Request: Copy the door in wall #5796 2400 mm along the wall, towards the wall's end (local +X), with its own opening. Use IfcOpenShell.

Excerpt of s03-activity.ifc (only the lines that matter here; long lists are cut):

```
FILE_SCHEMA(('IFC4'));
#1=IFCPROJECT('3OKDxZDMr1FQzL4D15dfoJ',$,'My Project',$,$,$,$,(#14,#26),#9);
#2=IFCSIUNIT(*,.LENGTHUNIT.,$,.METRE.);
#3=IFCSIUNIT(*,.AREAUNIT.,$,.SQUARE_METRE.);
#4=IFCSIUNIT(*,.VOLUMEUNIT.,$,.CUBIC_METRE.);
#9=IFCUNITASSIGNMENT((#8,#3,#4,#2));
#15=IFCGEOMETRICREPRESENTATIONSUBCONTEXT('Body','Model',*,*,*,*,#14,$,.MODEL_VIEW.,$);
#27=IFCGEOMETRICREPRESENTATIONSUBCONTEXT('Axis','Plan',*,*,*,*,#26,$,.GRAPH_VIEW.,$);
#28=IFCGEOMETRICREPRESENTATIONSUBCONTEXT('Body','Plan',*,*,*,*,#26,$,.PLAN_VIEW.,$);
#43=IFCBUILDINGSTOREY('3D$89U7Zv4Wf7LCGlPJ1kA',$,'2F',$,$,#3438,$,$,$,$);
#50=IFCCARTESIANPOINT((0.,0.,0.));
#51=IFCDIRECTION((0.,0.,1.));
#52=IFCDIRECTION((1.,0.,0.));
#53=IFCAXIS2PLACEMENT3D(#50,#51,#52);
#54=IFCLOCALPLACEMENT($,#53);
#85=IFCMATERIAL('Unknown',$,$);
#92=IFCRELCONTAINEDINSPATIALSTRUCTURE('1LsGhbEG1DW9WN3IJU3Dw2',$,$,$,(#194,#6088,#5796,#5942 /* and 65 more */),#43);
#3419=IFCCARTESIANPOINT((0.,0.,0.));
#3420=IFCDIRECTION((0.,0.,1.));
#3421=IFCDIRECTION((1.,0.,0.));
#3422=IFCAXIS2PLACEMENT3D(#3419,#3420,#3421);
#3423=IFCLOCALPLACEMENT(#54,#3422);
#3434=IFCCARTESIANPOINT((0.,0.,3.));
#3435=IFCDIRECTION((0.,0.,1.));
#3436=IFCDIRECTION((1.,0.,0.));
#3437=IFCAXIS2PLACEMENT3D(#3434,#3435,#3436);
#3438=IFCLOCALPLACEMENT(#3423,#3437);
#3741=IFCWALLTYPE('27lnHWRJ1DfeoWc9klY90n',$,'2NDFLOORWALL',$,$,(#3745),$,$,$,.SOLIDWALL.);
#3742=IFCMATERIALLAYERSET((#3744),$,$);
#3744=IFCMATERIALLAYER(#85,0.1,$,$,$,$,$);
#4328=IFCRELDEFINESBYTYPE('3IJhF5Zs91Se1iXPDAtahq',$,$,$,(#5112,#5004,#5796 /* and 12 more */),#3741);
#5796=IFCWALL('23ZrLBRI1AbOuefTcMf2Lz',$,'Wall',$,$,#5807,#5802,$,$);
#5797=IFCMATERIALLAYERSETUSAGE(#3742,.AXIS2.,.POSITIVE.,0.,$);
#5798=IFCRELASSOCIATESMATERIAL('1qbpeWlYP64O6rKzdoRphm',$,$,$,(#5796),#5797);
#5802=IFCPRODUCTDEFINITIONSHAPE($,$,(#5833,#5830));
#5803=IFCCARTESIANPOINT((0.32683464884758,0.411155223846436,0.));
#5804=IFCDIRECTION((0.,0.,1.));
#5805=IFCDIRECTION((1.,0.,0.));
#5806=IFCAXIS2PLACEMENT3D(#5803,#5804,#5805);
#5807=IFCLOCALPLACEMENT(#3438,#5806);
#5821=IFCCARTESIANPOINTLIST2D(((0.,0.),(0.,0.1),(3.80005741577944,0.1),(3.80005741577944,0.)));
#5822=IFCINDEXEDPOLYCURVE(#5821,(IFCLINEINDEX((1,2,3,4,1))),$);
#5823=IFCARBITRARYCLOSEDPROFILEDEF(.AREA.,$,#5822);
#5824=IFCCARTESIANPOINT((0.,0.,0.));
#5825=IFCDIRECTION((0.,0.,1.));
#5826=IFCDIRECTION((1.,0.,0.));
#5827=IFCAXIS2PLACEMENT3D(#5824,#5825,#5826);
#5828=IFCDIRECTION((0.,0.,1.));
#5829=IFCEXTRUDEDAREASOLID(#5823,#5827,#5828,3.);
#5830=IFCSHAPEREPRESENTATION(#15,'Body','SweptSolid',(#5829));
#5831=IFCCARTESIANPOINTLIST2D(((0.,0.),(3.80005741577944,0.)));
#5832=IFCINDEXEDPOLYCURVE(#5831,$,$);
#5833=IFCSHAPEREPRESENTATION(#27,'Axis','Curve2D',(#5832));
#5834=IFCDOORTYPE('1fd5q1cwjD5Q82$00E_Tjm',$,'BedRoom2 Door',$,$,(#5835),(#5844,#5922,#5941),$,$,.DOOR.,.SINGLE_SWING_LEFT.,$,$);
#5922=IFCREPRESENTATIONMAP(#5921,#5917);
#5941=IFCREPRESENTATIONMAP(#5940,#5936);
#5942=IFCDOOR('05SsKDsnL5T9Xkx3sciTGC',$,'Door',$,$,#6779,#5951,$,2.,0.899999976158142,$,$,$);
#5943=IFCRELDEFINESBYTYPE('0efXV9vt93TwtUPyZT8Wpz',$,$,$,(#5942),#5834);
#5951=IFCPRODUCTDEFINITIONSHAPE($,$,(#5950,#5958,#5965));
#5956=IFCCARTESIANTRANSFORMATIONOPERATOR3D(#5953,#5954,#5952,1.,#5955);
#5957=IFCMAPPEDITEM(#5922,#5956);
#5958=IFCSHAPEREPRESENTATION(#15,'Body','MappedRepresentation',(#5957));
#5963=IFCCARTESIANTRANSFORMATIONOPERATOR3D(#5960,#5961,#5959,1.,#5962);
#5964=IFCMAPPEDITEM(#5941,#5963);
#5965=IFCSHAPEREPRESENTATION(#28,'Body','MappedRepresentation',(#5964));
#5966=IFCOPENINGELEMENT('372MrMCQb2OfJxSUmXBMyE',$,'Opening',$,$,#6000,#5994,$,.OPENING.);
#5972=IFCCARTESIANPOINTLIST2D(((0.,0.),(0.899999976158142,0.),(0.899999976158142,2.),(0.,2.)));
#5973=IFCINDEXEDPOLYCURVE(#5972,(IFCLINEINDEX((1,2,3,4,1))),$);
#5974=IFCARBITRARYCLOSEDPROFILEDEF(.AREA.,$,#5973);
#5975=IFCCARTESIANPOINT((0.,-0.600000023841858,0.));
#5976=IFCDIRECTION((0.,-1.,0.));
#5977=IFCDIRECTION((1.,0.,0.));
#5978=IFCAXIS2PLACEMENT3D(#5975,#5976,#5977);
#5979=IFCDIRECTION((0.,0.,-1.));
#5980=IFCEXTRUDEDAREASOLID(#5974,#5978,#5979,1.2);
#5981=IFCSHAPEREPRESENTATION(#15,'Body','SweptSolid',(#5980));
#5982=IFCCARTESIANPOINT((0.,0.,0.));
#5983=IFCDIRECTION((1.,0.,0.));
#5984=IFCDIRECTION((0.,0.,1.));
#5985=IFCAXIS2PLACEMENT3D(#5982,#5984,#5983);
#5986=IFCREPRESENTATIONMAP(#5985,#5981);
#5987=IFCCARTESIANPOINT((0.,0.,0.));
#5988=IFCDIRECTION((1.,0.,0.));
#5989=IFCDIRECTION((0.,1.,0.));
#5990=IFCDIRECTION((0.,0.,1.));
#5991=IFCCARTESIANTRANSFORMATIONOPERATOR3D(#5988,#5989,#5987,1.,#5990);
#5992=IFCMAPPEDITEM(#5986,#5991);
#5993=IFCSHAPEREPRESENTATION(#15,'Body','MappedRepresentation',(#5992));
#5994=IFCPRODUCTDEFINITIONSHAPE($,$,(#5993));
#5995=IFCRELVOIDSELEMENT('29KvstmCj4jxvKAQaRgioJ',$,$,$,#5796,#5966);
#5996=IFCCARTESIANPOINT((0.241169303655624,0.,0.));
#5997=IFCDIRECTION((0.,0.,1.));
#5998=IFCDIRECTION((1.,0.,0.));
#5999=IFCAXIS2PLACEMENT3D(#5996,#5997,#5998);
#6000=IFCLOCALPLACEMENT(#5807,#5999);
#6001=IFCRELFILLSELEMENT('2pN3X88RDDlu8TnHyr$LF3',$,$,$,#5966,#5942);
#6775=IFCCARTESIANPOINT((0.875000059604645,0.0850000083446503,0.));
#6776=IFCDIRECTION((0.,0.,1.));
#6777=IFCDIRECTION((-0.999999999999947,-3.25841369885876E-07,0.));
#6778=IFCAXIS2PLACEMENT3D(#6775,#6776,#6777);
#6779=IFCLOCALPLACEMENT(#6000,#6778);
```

```python
import ifcopenshell
import ifcopenshell.api.feature
import ifcopenshell.api.geometry
import ifcopenshell.api.root
import ifcopenshell.geom
import ifcopenshell.util.element
import ifcopenshell.util.placement
import ifcopenshell.util.shape
import ifcopenshell.util.unit

model = ifcopenshell.open("s03-activity.ifc")
unit_scale = ifcopenshell.util.unit.calculate_unit_scale(model)
settings = ifcopenshell.geom.settings()


def volume(element):
    """Net volume in cubic metres, openings subtracted."""
    shape = ifcopenshell.geom.create_shape(settings, element)
    return ifcopenshell.util.shape.get_volume(shape.geometry)


door = model.by_guid("05SsKDsnL5T9Xkx3sciTGC")
opening = door.FillsVoids[0].RelatingOpeningElement
wall = opening.VoidsElements[0].RelatingBuildingElement
before = volume(wall)
shift = ifcopenshell.util.placement.get_local_placement(wall.ObjectPlacement)[:3, 0] * 2.4 / unit_scale

# copy_class copies the void relationship, type, container and properties, but no geometry.
new_opening = ifcopenshell.api.root.copy_class(model, product=opening)
new_opening.Representation = ifcopenshell.util.element.copy_deep(
    model, opening.Representation, exclude=["IfcGeometricRepresentationContext", "IfcRepresentationMap"]
)
new_door = ifcopenshell.api.root.copy_class(model, product=door)
new_door.Representation = ifcopenshell.util.element.copy_deep(
    model, door.Representation, exclude=["IfcGeometricRepresentationContext", "IfcRepresentationMap"]
)
ifcopenshell.api.feature.add_filling(model, opening=new_opening, element=new_door)

for old, new in ((opening, new_opening), (door, new_door)):
    matrix = ifcopenshell.util.placement.get_local_placement(old.ObjectPlacement)
    matrix[:3, 3] += shift
    ifcopenshell.api.geometry.edit_object_placement(model, product=new, matrix=matrix, is_si=False)

after = volume(wall)

print(f"wall volume {before:.3f} -> {after:.3f} m3")

model.write("s03-activity_edited.ifc")
```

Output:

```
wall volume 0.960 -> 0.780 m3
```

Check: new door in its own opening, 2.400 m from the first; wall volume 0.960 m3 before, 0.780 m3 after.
